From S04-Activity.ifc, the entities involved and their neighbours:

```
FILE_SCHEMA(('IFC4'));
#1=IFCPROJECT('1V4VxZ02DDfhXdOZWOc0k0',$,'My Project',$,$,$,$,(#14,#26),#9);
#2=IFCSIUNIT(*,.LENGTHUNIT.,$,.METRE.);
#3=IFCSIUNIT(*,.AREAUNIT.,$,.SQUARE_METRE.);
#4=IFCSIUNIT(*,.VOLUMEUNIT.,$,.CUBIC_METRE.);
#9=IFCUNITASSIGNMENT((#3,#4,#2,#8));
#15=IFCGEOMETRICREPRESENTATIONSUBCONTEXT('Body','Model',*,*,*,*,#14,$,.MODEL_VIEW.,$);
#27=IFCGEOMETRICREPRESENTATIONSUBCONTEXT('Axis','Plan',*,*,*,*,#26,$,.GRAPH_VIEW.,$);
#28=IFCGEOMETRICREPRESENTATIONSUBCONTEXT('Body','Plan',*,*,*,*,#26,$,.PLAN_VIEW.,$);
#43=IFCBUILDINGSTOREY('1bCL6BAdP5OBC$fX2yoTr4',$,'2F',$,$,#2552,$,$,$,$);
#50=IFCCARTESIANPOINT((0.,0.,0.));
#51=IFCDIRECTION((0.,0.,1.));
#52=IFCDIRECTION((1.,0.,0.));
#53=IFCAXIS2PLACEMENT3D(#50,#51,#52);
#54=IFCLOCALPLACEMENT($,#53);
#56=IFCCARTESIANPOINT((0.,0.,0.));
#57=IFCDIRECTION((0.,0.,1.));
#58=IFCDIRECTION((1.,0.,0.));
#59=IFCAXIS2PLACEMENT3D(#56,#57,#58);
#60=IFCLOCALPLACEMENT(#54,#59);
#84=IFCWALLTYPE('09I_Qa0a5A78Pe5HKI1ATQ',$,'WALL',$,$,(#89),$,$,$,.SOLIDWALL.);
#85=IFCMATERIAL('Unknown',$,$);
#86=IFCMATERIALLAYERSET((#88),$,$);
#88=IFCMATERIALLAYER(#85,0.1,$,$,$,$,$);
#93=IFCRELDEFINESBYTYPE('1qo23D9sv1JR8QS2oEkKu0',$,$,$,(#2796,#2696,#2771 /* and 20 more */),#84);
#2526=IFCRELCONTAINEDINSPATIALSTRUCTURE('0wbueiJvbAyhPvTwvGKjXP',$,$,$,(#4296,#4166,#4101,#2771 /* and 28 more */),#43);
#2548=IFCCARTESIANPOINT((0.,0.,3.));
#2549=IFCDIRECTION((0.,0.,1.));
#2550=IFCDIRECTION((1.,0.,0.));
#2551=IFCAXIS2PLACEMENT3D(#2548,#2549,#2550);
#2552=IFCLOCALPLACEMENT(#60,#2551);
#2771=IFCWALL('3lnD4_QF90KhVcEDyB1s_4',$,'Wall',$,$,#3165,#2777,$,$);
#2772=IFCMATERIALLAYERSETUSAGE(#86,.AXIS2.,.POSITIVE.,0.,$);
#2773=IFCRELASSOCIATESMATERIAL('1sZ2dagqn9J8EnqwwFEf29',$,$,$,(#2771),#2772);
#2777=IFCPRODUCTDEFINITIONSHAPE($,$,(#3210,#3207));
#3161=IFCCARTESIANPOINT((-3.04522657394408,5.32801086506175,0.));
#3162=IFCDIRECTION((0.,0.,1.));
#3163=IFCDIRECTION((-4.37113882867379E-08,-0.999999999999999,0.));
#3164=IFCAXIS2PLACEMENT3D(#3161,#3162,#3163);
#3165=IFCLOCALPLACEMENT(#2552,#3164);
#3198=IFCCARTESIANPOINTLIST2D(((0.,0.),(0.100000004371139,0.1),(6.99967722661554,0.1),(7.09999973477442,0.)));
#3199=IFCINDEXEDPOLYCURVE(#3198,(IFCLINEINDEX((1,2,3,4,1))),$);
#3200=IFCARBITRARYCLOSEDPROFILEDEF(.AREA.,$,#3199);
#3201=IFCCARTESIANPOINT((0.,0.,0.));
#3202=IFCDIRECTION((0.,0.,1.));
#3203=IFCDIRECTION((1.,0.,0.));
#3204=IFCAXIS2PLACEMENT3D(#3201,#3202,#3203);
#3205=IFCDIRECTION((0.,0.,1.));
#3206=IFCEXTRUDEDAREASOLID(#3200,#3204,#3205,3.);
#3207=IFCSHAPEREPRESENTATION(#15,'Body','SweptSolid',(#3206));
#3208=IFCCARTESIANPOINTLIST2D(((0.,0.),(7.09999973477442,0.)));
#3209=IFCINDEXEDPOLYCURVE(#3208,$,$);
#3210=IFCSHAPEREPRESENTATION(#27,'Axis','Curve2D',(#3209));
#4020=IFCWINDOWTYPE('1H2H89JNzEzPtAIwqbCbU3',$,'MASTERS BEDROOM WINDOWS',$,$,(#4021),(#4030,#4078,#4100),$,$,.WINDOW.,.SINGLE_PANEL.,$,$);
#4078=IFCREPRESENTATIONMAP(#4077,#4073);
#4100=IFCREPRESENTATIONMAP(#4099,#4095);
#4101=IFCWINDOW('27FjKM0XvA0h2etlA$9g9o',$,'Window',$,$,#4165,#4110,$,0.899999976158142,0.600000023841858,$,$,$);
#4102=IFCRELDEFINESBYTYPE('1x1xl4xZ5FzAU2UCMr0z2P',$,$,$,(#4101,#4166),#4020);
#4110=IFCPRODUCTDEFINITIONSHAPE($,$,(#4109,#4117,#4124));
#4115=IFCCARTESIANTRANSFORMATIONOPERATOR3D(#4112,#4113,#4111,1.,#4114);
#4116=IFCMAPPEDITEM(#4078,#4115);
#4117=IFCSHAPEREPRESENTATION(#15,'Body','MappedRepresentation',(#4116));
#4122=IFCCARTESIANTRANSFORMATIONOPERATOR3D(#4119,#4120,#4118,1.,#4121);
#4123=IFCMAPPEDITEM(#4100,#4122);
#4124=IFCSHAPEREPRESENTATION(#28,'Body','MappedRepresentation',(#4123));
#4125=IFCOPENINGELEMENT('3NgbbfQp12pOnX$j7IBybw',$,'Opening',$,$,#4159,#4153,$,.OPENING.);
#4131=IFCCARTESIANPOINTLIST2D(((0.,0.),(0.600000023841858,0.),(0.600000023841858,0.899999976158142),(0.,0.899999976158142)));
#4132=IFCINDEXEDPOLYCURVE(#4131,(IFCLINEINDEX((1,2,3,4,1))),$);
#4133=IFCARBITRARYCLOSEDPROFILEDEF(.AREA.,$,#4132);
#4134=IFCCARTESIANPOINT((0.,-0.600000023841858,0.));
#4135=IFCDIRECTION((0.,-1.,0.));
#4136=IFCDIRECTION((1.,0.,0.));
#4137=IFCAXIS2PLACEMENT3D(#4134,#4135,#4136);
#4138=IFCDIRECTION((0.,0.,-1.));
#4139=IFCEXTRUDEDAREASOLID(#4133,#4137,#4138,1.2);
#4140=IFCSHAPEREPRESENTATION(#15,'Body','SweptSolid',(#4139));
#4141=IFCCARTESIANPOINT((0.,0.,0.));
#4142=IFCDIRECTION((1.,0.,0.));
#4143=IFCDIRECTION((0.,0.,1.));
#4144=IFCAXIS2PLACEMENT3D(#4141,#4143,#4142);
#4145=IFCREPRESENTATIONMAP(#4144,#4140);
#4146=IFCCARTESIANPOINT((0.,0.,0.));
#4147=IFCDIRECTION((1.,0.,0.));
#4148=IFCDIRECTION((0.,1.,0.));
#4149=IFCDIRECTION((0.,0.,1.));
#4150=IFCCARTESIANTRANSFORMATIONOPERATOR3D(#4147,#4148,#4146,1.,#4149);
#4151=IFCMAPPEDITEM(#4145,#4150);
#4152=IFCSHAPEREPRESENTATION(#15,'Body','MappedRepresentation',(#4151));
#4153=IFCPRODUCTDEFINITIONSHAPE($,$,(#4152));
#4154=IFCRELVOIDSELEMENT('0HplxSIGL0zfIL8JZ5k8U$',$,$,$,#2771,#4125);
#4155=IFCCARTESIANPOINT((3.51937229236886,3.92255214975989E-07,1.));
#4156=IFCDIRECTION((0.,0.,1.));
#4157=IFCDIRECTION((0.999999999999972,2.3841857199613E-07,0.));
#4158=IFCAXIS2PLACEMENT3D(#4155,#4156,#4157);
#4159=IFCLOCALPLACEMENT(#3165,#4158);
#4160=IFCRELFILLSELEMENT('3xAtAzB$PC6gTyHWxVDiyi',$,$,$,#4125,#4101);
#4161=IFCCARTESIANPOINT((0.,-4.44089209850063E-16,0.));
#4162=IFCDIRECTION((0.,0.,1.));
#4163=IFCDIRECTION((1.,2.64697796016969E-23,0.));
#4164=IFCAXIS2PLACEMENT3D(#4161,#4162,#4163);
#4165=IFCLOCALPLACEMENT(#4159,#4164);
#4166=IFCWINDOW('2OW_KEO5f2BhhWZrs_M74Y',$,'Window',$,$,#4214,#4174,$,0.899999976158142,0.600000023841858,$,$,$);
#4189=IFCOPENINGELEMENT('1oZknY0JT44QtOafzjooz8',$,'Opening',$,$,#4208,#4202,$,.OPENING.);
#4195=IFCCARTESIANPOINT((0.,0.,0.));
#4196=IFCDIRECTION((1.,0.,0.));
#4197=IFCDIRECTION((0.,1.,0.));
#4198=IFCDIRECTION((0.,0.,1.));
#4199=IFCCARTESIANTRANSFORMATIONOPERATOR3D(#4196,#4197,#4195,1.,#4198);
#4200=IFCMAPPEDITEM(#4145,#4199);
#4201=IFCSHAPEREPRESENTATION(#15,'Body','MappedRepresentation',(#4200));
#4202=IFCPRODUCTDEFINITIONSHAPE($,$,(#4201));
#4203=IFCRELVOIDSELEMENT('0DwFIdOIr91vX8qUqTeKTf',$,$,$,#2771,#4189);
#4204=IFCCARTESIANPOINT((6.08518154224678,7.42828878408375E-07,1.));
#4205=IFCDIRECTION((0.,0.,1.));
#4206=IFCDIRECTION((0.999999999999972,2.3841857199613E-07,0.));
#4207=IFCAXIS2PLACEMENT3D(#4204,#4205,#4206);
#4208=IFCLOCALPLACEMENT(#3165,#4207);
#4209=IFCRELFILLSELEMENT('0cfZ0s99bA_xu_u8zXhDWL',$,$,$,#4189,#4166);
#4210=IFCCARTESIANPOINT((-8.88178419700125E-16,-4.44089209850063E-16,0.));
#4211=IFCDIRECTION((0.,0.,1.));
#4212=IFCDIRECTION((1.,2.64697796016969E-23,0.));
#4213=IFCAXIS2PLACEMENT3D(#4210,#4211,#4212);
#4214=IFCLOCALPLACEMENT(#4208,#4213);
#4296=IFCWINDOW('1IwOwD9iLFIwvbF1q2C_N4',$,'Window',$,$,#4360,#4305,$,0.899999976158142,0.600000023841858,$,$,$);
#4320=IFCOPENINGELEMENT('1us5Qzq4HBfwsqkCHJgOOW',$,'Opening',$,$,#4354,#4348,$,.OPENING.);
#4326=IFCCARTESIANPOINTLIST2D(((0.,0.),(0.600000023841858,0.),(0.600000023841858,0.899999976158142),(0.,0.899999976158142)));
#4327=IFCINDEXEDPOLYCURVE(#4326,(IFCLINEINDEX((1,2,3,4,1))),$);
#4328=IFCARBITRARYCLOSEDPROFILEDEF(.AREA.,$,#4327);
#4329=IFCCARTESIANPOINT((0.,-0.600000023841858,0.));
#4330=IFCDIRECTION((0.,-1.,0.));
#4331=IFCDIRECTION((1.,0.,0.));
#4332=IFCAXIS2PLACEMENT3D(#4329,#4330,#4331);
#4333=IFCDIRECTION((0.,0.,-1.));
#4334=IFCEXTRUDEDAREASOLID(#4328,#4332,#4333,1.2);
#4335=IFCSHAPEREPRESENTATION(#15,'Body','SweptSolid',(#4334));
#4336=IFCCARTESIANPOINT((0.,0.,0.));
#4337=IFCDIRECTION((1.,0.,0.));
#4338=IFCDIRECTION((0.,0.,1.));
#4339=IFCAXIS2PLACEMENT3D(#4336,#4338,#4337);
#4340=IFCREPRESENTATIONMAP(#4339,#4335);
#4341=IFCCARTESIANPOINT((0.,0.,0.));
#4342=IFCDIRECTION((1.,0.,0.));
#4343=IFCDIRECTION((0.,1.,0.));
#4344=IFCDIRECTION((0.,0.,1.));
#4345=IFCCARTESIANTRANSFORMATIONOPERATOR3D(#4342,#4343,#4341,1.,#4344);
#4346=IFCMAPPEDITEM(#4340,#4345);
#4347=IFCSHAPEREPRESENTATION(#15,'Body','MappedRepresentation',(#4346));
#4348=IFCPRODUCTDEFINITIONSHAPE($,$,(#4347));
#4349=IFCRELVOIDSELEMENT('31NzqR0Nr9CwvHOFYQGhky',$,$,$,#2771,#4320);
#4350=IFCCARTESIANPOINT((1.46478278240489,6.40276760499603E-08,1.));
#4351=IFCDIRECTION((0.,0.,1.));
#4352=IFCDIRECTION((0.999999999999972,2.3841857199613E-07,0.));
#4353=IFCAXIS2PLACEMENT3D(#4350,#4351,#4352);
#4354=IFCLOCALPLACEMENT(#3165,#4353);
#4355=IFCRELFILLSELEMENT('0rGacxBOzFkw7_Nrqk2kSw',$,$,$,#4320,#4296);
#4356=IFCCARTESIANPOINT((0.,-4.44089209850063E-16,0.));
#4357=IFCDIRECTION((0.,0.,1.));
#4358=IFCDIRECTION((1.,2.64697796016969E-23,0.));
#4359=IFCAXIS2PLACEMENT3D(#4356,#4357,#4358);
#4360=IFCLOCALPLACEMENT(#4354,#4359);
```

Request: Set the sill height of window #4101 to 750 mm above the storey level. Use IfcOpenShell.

```python
import numpy as np
import ifcopenshell
import ifcopenshell.api.geometry
import ifcopenshell.geom
import ifcopenshell.util.element
import ifcopenshell.util.placement
import ifcopenshell.util.shape
import ifcopenshell.util.unit

model = ifcopenshell.open("S04-Activity.ifc")
unit_scale = ifcopenshell.util.unit.calculate_unit_scale(model)

window = model.by_id(4101)
opening = window.FillsVoids[0].RelatingOpeningElement
storey = ifcopenshell.util.element.get_container(window, ifc_class="IfcBuildingStorey")
level = ifcopenshell.util.placement.get_local_placement(storey.ObjectPlacement)[2, 3]

# The opening's origin need not be at the sill, so measure its lowest point.
shape = ifcopenshell.geom.create_shape(ifcopenshell.geom.settings(), opening)
bottom = ifcopenshell.util.shape.get_shape_bottom_elevation(shape, shape.geometry) / unit_scale
dz = level + 0.75 / unit_scale - bottom

shift = np.array([0.0, 0.0, dz])
# The window is placed relative to its opening, so it follows when the opening moves.
matrix = ifcopenshell.util.placement.get_local_placement(opening.ObjectPlacement)
matrix[:3, 3] += shift
ifcopenshell.api.geometry.edit_object_placement(
    model, product=opening, matrix=matrix, is_si=False, should_transform_children=True
)

print(f"moved by {dz * unit_scale:+.3f} m")

model.write("S04-Activity_rev.ifc")
```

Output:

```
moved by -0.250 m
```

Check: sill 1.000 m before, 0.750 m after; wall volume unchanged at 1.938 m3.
